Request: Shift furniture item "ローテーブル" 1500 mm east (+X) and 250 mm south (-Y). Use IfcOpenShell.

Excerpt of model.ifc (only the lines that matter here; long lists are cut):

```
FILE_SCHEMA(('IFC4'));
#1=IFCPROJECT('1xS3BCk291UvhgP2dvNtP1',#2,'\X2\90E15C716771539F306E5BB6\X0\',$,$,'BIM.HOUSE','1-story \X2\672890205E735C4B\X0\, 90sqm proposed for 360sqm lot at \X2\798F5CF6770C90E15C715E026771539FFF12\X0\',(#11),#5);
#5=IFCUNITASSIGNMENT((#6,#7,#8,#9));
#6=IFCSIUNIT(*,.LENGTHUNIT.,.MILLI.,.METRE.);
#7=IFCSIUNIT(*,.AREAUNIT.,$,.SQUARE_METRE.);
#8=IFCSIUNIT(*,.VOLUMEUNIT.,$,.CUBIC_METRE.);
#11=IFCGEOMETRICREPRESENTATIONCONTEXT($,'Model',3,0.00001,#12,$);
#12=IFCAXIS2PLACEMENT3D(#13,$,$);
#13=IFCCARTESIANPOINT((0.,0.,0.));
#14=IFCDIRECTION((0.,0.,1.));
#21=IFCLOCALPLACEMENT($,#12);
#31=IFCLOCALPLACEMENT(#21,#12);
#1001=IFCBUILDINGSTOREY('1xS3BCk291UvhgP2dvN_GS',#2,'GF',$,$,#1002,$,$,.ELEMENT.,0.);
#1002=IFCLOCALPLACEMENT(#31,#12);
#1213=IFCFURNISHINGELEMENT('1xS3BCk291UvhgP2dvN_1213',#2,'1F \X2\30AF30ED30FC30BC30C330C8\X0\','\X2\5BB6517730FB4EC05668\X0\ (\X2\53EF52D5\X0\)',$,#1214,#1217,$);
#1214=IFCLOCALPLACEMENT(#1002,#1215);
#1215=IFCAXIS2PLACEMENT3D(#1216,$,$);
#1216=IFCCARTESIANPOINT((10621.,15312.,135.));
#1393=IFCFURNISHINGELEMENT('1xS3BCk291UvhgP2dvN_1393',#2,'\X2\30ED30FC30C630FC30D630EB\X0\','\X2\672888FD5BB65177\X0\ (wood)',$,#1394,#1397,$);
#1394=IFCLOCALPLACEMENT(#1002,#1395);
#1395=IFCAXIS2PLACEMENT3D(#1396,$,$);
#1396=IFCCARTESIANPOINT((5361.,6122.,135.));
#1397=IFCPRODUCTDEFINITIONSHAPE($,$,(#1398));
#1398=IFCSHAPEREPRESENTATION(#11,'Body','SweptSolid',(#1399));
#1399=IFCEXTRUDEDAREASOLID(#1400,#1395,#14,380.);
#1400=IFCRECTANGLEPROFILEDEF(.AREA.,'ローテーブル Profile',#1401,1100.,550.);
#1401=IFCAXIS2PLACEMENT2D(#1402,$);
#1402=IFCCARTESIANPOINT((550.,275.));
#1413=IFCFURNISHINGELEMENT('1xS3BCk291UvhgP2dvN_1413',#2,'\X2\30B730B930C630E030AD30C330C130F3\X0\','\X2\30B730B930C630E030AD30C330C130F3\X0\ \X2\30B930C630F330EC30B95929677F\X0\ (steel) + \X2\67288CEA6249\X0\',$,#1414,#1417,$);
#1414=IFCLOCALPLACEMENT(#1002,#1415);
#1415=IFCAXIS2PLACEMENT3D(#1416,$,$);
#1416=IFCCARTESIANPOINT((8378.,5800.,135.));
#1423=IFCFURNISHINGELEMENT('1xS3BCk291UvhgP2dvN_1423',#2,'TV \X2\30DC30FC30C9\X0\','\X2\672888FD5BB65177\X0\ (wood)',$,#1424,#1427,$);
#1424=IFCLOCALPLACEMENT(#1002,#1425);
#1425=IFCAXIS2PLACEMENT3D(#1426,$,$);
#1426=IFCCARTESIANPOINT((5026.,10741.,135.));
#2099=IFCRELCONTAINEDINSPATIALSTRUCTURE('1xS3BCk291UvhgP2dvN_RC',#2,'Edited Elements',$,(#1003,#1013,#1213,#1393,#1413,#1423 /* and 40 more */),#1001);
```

```python
import ifcopenshell
import ifcopenshell.api.geometry
import ifcopenshell.util.placement
import ifcopenshell.util.unit

model = ifcopenshell.open("model.ifc")
unit_scale = ifcopenshell.util.unit.calculate_unit_scale(model)

item = model.by_guid("1xS3BCk291UvhgP2dvN_1393")
matrix = ifcopenshell.util.placement.get_local_placement(item.ObjectPlacement)
matrix[0, 3] += 1.5 / unit_scale
matrix[1, 3] -= 0.25 / unit_scale
ifcopenshell.api.geometry.edit_object_placement(model, product=item, matrix=matrix, is_si=False)

print(ifcopenshell.util.placement.get_local_placement(item.ObjectPlacement).round(3) + 0.0)

model.write("model_rev.ifc")
```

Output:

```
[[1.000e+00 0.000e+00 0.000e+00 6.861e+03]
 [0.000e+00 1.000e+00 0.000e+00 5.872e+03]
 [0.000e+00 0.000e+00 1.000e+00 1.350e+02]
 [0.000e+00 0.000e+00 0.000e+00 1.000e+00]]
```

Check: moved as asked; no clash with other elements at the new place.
